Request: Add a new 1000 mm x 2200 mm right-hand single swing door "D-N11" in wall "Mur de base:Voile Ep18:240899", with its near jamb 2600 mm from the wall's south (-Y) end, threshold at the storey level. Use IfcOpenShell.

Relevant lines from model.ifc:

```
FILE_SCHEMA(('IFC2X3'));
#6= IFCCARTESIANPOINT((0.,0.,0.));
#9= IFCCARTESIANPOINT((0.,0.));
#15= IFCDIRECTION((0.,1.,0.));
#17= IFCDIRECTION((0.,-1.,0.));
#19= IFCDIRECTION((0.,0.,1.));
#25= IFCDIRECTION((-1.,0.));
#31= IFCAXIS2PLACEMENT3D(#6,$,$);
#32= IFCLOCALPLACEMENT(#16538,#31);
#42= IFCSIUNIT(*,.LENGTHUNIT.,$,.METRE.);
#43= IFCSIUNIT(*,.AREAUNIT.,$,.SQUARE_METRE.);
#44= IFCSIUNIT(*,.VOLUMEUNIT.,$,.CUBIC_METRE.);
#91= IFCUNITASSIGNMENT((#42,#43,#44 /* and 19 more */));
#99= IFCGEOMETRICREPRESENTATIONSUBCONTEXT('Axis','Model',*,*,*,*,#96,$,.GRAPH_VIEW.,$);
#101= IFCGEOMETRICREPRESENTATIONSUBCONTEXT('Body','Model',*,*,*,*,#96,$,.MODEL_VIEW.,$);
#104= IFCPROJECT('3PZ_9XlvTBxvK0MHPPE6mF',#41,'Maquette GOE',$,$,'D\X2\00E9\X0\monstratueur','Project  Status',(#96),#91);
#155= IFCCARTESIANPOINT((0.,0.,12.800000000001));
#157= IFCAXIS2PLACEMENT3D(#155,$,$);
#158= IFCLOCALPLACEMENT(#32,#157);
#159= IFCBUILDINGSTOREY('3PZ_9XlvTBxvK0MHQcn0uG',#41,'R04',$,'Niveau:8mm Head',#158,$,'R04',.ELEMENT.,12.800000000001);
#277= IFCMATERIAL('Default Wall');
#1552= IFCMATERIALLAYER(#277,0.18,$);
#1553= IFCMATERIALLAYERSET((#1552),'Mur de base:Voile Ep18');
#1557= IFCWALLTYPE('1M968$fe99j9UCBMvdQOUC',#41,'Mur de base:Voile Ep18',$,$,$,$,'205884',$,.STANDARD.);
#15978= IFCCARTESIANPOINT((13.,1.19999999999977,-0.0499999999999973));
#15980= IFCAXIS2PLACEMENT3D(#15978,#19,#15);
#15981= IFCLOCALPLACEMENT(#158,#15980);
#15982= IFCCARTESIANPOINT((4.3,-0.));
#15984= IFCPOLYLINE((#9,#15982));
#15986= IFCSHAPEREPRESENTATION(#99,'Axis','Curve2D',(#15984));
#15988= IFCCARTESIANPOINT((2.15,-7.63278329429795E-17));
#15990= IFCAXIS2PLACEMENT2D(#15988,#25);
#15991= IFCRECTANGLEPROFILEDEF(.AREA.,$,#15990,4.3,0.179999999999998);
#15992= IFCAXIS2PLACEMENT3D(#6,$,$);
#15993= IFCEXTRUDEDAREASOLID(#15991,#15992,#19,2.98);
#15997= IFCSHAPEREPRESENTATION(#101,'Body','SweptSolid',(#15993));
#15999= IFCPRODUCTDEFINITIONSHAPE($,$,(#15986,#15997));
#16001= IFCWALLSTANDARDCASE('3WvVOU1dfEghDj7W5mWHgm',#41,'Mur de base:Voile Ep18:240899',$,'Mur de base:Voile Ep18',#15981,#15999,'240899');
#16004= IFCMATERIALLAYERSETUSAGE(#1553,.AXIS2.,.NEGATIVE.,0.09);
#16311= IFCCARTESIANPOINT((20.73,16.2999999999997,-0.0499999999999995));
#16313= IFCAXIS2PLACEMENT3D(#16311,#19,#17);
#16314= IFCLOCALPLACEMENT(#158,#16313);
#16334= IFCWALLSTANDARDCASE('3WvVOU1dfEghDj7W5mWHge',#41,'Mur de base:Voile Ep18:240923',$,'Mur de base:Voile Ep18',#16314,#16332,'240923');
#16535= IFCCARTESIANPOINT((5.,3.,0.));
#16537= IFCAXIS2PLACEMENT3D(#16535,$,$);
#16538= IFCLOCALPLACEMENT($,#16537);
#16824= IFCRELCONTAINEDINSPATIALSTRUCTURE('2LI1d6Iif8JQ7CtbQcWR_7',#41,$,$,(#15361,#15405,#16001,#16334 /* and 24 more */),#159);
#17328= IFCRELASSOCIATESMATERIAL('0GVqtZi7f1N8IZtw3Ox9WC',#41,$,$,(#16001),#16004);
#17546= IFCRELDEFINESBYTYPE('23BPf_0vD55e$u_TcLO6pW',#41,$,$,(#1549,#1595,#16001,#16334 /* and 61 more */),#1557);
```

```python
import numpy as np
import ifcopenshell
import ifcopenshell.api.feature
import ifcopenshell.api.geometry
import ifcopenshell.api.root
import ifcopenshell.api.spatial
import ifcopenshell.api.type
import ifcopenshell.geom
import ifcopenshell.util.element
import ifcopenshell.util.placement
import ifcopenshell.util.representation
import ifcopenshell.util.shape
import ifcopenshell.util.unit

model = ifcopenshell.open("model.ifc")
unit_scale = ifcopenshell.util.unit.calculate_unit_scale(model)
settings = ifcopenshell.geom.settings()


def volume(element):
    """Net volume in cubic metres, openings subtracted."""
    shape = ifcopenshell.geom.create_shape(settings, element)
    return ifcopenshell.util.shape.get_volume(shape.geometry)


wall = model.by_id(16001)
storey = ifcopenshell.util.element.get_container(wall, ifc_class="IfcBuildingStorey")
context = ifcopenshell.util.representation.get_context(model, "Model", "Body", "MODEL_VIEW")
before = volume(wall)

width, height, from_end, sill = 1, 2.2, 2.6, 0.0  # metres

# The wall runs along its own X axis, and the end named is its -X end.
wall_shape = ifcopenshell.geom.create_shape(settings, wall)
x, y, z = ifcopenshell.util.shape.get_vertices(wall_shape.geometry).T
start = x.min() + from_end
face, thickness = float(y.min()), float(y.max() - y.min())
wall_matrix = ifcopenshell.util.placement.get_local_placement(wall.ObjectPlacement)
level = ifcopenshell.util.placement.get_local_placement(storey.ObjectPlacement)[2, 3]


def in_wall(x, y):
    """Placement at x, y metres in the wall's axes, at sill height."""
    matrix = wall_matrix.copy()
    matrix[:, 3] = wall_matrix @ np.array([x / unit_scale, y / unit_scale, 0.0, 1.0])
    matrix[2, 3] = level + sill / unit_scale
    return matrix


# Opening: a box that overshoots both wall faces by 50 mm.
opening = ifcopenshell.api.root.create_entity(model, ifc_class="IfcOpeningElement")
box = ifcopenshell.api.geometry.add_wall_representation(
    model, context=context, length=width, height=height, thickness=thickness + 0.1
)
ifcopenshell.api.geometry.assign_representation(model, product=opening, representation=box)
ifcopenshell.api.geometry.edit_object_placement(model, product=opening, matrix=in_wall(start, face - 0.05), is_si=False)
ifcopenshell.api.feature.add_feature(model, feature=opening, element=wall)

door = ifcopenshell.api.root.create_entity(model, ifc_class="IfcDoor", name="D-N11")
door.OverallWidth, door.OverallHeight = width / unit_scale, height / unit_scale
body = ifcopenshell.api.geometry.add_door_representation(
    model,
    context=context,
    overall_width=door.OverallWidth,
    overall_height=door.OverallHeight,
    operation_type="SINGLE_SWING_RIGHT",
    lining_properties={"LiningDepth": thickness / unit_scale, "ThresholdDepth": thickness / unit_scale},
)
ifcopenshell.api.geometry.assign_representation(model, product=door, representation=body)
ifcopenshell.api.spatial.assign_container(model, products=[door], relating_structure=storey)
fills = ifcopenshell.api.feature.add_filling(model, opening=opening, element=door)
fills.OwnerHistory = door.OwnerHistory  # required in IFC2X3

# IFC2X3 keeps the operation on the door style.
style = ifcopenshell.api.root.create_entity(model, ifc_class="IfcDoorStyle", name="D-N11")
style.OperationType, style.ConstructionType = "SINGLE_SWING_RIGHT", "NOTDEFINED"
style.ParameterTakesPrecedence = style.Sizeable = False
ifcopenshell.api.type.assign_type(model, related_objects=[door], relating_type=style)

# The lining spans the wall, so the door starts at the wall face.
ifcopenshell.api.geometry.edit_object_placement(model, product=door, matrix=in_wall(start, face), is_si=False)

after = volume(wall)

print(f"wall volume {before:.3f} -> {after:.3f} m3")

model.write("model_updated.ifc")
```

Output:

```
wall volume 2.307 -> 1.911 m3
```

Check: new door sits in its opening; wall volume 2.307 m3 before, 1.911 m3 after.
